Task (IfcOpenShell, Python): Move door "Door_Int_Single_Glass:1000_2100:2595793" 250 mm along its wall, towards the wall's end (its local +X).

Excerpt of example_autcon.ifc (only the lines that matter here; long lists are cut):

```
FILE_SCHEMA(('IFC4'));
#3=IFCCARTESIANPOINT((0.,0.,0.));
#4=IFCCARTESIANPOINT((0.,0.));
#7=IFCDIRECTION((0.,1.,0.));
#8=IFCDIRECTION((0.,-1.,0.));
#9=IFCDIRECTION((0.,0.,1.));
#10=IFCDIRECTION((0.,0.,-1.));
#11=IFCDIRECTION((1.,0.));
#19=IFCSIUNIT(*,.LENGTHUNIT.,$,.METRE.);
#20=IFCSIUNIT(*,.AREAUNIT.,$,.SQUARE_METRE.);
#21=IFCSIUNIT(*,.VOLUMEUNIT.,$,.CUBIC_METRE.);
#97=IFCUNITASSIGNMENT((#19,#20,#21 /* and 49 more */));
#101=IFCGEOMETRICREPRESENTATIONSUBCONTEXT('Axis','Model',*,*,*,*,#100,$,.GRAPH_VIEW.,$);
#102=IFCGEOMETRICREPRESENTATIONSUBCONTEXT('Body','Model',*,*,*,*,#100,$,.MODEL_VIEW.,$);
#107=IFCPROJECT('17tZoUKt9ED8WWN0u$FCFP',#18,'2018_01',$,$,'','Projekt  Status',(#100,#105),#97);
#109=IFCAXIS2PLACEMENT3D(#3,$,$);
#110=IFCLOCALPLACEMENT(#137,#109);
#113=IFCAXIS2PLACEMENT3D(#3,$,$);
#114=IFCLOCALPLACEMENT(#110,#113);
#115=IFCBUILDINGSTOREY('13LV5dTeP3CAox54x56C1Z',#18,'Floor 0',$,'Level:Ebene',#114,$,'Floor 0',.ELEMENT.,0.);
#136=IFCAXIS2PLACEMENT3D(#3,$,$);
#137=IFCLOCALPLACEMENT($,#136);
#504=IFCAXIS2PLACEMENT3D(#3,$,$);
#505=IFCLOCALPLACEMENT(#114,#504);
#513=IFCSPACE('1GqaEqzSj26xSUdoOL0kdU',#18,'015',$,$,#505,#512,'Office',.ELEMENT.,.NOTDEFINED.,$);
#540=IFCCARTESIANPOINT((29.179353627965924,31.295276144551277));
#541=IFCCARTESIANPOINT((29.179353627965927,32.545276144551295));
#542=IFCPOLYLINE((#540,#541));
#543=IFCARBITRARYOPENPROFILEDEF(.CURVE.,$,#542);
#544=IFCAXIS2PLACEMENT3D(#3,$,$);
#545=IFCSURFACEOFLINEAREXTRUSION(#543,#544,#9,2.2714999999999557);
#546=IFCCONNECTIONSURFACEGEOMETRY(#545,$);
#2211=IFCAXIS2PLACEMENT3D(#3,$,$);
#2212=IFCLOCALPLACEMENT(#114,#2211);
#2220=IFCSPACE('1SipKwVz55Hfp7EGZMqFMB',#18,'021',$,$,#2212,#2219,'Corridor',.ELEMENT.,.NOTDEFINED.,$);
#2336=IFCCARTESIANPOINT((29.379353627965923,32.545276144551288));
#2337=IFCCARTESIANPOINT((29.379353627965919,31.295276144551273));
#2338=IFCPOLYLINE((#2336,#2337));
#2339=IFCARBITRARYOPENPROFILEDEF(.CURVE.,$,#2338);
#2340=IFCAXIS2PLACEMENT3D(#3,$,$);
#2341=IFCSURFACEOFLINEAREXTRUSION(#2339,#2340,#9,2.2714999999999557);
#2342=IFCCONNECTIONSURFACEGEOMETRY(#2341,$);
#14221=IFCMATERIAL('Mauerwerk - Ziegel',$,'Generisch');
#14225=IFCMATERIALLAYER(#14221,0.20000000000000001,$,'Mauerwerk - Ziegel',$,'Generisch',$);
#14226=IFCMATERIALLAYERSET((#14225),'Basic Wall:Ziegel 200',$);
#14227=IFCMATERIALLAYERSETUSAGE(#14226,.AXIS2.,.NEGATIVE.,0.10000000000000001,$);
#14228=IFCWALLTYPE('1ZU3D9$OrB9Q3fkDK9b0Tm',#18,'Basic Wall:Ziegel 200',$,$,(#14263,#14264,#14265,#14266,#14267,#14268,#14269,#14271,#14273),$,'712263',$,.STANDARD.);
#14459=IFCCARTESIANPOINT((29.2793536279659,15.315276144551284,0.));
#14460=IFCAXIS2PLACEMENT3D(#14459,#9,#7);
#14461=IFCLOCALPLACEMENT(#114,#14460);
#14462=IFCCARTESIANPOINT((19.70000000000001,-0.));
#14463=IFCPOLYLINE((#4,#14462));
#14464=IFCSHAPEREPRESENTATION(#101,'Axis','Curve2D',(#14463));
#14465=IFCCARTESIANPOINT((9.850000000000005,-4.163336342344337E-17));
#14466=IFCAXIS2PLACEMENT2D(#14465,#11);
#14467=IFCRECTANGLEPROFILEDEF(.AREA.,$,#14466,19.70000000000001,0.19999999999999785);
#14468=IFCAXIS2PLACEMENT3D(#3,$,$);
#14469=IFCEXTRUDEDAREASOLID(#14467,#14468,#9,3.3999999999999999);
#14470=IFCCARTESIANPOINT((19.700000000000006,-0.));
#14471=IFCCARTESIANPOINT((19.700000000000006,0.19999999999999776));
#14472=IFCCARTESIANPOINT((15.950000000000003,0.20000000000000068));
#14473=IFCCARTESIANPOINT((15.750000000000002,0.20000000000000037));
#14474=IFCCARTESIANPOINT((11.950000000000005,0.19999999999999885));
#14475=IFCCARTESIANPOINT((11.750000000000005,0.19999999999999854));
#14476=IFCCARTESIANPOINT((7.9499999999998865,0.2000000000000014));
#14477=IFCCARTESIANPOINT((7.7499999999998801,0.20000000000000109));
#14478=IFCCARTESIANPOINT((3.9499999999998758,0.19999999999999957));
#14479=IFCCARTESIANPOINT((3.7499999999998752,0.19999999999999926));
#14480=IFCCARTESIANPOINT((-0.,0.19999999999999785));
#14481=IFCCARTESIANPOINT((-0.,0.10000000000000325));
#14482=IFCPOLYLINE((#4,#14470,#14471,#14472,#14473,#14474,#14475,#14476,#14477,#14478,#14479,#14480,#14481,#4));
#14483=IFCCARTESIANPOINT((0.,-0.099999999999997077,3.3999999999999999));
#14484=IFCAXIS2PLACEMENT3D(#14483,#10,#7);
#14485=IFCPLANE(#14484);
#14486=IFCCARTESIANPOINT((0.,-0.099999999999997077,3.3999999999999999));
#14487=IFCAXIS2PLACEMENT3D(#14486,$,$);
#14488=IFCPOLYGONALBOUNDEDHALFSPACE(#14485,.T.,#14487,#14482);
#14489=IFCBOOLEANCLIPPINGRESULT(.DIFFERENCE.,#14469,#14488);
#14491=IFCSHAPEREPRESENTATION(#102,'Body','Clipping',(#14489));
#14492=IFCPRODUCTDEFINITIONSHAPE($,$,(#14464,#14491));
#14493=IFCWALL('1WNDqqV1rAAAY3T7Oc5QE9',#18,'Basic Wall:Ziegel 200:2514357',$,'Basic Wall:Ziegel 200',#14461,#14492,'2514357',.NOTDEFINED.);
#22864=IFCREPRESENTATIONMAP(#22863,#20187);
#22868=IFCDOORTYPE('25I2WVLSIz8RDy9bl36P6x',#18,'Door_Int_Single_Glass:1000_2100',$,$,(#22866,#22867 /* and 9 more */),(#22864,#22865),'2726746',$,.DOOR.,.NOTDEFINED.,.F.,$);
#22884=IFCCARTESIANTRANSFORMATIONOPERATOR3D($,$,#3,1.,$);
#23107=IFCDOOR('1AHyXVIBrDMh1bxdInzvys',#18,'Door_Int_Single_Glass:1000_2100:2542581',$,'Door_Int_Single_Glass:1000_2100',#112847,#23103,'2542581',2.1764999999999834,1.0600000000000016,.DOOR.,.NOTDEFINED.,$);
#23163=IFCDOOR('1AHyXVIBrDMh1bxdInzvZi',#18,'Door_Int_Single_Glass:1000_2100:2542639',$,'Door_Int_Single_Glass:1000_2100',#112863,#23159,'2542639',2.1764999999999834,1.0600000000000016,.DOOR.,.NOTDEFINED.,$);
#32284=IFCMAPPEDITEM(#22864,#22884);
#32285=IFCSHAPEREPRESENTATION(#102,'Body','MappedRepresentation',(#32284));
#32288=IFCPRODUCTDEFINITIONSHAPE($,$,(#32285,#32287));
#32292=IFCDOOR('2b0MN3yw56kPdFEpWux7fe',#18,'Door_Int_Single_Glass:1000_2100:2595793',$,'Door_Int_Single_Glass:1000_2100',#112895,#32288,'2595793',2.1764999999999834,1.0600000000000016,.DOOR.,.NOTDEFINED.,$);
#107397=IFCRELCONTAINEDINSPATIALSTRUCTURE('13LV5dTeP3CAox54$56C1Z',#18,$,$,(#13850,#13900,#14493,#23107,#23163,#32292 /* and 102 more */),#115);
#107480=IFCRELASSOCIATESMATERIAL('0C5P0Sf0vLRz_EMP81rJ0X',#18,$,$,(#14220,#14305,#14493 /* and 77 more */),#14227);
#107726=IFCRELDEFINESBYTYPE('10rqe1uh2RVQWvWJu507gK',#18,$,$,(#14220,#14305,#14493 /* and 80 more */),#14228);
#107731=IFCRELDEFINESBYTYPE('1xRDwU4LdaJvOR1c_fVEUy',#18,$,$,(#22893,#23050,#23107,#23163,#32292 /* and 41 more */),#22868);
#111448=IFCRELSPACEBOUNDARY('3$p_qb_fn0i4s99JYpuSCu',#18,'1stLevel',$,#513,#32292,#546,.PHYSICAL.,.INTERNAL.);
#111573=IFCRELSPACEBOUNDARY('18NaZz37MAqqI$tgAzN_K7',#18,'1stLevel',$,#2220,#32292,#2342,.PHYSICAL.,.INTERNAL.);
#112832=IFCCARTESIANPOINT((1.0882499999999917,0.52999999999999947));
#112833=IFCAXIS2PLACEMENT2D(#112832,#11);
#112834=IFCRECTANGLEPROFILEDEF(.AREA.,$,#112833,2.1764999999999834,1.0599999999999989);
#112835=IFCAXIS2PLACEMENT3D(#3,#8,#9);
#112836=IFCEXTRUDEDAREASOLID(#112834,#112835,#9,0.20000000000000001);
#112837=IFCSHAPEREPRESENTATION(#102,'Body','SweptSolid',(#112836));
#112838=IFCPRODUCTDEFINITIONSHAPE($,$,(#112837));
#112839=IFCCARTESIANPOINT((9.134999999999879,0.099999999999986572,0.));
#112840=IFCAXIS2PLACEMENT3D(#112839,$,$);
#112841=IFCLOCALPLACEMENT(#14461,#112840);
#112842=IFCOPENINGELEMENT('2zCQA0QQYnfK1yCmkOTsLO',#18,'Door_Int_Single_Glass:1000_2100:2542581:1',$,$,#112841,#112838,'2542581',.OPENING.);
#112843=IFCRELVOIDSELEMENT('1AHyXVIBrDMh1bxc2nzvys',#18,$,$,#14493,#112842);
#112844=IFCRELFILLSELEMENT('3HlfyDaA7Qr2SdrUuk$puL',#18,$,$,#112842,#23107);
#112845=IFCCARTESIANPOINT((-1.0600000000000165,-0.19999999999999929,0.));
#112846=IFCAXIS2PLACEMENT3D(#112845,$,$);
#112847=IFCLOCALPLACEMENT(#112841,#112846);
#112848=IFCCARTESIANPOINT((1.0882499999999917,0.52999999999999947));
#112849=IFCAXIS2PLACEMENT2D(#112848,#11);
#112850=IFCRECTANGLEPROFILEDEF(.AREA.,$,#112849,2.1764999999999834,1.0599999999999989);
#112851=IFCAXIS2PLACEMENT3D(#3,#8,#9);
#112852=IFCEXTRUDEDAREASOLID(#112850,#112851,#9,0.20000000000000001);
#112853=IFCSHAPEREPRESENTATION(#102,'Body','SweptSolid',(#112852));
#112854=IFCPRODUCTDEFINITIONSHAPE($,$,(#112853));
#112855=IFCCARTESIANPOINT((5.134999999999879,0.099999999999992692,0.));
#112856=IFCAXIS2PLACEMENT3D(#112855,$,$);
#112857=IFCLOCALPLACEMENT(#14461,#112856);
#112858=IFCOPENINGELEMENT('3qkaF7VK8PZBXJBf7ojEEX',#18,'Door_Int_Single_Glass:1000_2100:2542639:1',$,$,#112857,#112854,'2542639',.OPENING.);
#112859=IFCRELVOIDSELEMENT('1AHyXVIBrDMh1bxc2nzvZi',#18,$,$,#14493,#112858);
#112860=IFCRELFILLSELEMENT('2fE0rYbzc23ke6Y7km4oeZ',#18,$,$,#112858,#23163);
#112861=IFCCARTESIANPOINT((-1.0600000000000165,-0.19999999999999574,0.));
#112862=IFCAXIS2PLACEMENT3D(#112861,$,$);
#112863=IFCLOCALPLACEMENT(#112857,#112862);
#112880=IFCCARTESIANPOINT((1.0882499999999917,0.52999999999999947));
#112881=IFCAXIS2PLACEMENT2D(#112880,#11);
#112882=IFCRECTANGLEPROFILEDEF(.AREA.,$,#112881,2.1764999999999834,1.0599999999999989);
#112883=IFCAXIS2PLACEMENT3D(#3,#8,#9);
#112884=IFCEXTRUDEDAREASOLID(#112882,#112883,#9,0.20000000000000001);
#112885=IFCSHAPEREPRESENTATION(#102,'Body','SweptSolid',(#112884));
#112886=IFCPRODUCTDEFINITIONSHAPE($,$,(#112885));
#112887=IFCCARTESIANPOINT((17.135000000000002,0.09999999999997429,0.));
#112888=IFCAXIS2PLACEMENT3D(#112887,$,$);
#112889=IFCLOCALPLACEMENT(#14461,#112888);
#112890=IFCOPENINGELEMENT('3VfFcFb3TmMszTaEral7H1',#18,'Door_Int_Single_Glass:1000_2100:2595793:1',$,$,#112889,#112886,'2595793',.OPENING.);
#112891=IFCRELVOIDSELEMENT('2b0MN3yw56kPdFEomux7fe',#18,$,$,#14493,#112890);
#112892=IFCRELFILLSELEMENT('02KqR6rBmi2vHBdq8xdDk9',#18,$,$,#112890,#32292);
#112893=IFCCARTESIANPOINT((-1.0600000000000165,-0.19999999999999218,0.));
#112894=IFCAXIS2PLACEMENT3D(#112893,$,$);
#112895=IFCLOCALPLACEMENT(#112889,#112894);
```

```python
import numpy as np
import ifcopenshell
import ifcopenshell.api.geometry
import ifcopenshell.util.placement

model = ifcopenshell.open("example_autcon.ifc")

door = model.by_guid("2b0MN3yw56kPdFEpWux7fe")
opening = door.FillsVoids[0].RelatingOpeningElement
wall = opening.VoidsElements[0].RelatingBuildingElement

wall_matrix = ifcopenshell.util.placement.get_local_placement(wall.ObjectPlacement)
shift = wall_matrix[:3, 0] * 0.25
before = ifcopenshell.util.placement.get_local_placement(door.ObjectPlacement)[:3, 3].copy()

# The door is placed relative to its opening, so it follows when the opening moves.
matrix = ifcopenshell.util.placement.get_local_placement(opening.ObjectPlacement)
matrix[:3, 3] += shift
ifcopenshell.api.geometry.edit_object_placement(
    model, product=opening, matrix=matrix, is_si=False, should_transform_children=True
)

# Space boundary surfaces are stored in each space's coordinates; move them too.
for rel in door.ProvidesBoundaries:
    if not rel.ConnectionGeometry:
        continue
    surface = rel.ConnectionGeometry.SurfaceOnRelatingElement
    space_matrix = ifcopenshell.util.placement.get_local_placement(rel.RelatingSpace.ObjectPlacement)
    point = np.array(surface.Position.Location.Coordinates) + space_matrix[:3, :3].T @ shift
    surface.Position = model.createIfcAxis2Placement3D(
        model.createIfcCartesianPoint(point.tolist()), surface.Position.Axis, surface.Position.RefDirection
    )

after = ifcopenshell.util.placement.get_local_placement(door.ObjectPlacement)[:3, 3]
print("door moved by", (after - before).round(3) + 0.0)

model.write("example_autcon_rev.ifc")
```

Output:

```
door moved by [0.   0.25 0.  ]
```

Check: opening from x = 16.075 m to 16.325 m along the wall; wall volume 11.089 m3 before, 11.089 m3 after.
